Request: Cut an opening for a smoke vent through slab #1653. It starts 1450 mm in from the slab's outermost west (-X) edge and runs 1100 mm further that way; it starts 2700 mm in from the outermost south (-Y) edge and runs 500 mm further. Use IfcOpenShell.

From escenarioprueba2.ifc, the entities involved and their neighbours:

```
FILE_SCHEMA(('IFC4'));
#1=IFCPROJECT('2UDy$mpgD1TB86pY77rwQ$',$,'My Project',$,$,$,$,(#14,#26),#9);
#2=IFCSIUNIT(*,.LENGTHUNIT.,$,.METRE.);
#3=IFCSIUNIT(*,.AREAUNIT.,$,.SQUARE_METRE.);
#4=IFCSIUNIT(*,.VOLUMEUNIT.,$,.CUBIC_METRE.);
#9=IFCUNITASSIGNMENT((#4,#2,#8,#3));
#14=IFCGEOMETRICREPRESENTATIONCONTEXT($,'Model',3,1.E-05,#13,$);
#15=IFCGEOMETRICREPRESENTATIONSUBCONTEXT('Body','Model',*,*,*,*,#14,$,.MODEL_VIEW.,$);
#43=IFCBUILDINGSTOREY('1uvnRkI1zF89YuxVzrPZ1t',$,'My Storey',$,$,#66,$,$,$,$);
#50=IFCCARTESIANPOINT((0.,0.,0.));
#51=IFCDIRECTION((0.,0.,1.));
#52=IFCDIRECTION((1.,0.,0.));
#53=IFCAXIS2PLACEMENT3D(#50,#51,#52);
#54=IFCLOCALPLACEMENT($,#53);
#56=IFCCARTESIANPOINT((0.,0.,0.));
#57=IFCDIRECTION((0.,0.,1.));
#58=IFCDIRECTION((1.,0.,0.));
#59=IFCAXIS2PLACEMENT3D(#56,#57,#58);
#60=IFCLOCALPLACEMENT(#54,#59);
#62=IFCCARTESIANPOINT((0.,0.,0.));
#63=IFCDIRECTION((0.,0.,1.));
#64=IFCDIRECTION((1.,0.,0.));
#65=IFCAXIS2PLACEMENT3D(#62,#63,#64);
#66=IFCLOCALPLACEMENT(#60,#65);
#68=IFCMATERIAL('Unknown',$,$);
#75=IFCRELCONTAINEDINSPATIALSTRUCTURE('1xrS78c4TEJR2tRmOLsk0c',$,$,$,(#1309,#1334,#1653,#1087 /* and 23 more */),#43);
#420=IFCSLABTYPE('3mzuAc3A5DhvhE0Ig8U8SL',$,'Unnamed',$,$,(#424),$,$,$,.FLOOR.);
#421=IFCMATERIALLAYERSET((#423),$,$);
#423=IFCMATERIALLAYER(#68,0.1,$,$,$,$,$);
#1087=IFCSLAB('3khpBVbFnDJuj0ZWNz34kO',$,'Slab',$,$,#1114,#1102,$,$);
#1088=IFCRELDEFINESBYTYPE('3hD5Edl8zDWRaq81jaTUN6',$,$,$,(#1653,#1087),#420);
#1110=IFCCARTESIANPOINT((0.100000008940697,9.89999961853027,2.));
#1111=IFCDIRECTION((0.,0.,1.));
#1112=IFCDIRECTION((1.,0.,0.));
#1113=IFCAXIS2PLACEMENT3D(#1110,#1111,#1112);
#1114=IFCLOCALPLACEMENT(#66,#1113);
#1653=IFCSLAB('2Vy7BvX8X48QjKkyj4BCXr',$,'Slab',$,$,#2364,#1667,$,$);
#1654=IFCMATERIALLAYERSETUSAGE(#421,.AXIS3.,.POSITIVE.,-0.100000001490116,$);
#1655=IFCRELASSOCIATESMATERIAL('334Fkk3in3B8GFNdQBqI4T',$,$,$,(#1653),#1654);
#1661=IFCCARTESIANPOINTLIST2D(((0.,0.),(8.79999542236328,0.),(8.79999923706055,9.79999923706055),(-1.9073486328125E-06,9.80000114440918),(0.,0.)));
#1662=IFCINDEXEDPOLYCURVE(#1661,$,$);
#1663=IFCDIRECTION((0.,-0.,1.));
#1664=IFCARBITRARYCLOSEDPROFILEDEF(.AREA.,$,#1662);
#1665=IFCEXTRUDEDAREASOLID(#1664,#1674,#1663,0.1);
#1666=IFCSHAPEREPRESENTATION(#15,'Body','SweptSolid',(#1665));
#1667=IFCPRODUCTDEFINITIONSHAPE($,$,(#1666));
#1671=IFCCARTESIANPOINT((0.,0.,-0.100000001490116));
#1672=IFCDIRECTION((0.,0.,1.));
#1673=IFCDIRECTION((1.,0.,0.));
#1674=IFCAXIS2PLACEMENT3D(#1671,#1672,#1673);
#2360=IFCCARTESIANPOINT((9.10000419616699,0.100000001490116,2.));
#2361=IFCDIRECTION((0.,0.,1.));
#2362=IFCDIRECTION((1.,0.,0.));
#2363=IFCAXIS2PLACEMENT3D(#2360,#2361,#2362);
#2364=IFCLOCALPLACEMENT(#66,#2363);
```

```python
import numpy as np
import ifcopenshell
import ifcopenshell.api.feature
import ifcopenshell.api.geometry
import ifcopenshell.api.root
import ifcopenshell.geom
import ifcopenshell.util.placement
import ifcopenshell.util.representation
import ifcopenshell.util.shape
import ifcopenshell.util.unit

model = ifcopenshell.open("escenarioprueba2.ifc")
unit_scale = ifcopenshell.util.unit.calculate_unit_scale(model)
settings = ifcopenshell.geom.settings()


def volume(element):
    """Net volume in cubic metres, openings subtracted."""
    shape = ifcopenshell.geom.create_shape(settings, element)
    return ifcopenshell.util.shape.get_volume(shape.geometry)


slab = model.by_guid("2Vy7BvX8X48QjKkyj4BCXr")
before = volume(slab)

# Extent in the slab's own axes, in metres. The edges named are its -X and -Y sides.
slab_shape = ifcopenshell.geom.create_shape(settings, slab)
vertices = ifcopenshell.util.shape.get_vertices(slab_shape.geometry)
x_min, y_min, bottom = vertices.min(axis=0)
top = vertices[:, 2].max()

opening = ifcopenshell.api.root.create_entity(model, ifc_class="IfcOpeningElement", name="Smoke vent opening", predefined_type="OPENING")
context = ifcopenshell.util.representation.get_context(model, "Model", "Body", "MODEL_VIEW")
width, depth = 1.1, 0.5
outline = [(0.0, 0.0), (width, 0.0), (width, depth), (0.0, depth), (0.0, 0.0)]
# Overshoot both faces by 50 mm so the cut is clean.
shape = ifcopenshell.api.geometry.add_slab_representation(
    model, context=context, depth=top - bottom + 0.1, polyline=outline
)
ifcopenshell.api.geometry.assign_representation(model, product=opening, representation=shape)

matrix = ifcopenshell.util.placement.get_local_placement(slab.ObjectPlacement)
matrix[:, 3] = matrix @ np.append(np.array([x_min + 1.45, y_min + 2.7, bottom - 0.05]) / unit_scale, 1.0)
ifcopenshell.api.geometry.edit_object_placement(model, product=opening, matrix=matrix, is_si=False)
ifcopenshell.api.feature.add_feature(model, feature=opening, element=slab)

after = volume(slab)

print(f"slab volume {before:.3f} -> {after:.3f} m3")

model.write("escenarioprueba2_updated.ifc")
```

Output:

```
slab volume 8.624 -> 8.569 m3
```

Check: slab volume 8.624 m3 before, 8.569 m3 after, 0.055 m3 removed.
